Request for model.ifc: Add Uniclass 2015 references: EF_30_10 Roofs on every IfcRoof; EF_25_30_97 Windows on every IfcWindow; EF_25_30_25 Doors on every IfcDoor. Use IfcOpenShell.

First a look at what the model holds.

```python
import ifcopenshell

model = ifcopenshell.open("model.ifc")
print(model.schema)
print("classifications:", [c.Name for c in model.by_type("IfcClassification")])
for ifc_class in ("IfcDoor", "IfcRoof", "IfcStair", "IfcWall", "IfcWindow"):
    print(ifc_class, len(model.by_type(ifc_class)))
```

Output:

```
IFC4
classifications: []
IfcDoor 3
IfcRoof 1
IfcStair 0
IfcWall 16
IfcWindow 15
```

```python
import ifcopenshell
import ifcopenshell.api.classification

model = ifcopenshell.open("model.ifc")

system = ifcopenshell.api.classification.add_classification(model, classification="Uniclass 2015")

codes = {
    "IfcRoof": ("EF_30_10", "Roofs"),
    "IfcWindow": ("EF_25_30_97", "Windows"),
    "IfcDoor": ("EF_25_30_25", "Doors"),
}
for ifc_class, (code, name) in codes.items():
    products = model.by_type(ifc_class)
    ifcopenshell.api.classification.add_reference(
        model, products=products, classification=system, identification=code, name=name
    )
    print(code, len(products))

model.write("model_rev.ifc")
```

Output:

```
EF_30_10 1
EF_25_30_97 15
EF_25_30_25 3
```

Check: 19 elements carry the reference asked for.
